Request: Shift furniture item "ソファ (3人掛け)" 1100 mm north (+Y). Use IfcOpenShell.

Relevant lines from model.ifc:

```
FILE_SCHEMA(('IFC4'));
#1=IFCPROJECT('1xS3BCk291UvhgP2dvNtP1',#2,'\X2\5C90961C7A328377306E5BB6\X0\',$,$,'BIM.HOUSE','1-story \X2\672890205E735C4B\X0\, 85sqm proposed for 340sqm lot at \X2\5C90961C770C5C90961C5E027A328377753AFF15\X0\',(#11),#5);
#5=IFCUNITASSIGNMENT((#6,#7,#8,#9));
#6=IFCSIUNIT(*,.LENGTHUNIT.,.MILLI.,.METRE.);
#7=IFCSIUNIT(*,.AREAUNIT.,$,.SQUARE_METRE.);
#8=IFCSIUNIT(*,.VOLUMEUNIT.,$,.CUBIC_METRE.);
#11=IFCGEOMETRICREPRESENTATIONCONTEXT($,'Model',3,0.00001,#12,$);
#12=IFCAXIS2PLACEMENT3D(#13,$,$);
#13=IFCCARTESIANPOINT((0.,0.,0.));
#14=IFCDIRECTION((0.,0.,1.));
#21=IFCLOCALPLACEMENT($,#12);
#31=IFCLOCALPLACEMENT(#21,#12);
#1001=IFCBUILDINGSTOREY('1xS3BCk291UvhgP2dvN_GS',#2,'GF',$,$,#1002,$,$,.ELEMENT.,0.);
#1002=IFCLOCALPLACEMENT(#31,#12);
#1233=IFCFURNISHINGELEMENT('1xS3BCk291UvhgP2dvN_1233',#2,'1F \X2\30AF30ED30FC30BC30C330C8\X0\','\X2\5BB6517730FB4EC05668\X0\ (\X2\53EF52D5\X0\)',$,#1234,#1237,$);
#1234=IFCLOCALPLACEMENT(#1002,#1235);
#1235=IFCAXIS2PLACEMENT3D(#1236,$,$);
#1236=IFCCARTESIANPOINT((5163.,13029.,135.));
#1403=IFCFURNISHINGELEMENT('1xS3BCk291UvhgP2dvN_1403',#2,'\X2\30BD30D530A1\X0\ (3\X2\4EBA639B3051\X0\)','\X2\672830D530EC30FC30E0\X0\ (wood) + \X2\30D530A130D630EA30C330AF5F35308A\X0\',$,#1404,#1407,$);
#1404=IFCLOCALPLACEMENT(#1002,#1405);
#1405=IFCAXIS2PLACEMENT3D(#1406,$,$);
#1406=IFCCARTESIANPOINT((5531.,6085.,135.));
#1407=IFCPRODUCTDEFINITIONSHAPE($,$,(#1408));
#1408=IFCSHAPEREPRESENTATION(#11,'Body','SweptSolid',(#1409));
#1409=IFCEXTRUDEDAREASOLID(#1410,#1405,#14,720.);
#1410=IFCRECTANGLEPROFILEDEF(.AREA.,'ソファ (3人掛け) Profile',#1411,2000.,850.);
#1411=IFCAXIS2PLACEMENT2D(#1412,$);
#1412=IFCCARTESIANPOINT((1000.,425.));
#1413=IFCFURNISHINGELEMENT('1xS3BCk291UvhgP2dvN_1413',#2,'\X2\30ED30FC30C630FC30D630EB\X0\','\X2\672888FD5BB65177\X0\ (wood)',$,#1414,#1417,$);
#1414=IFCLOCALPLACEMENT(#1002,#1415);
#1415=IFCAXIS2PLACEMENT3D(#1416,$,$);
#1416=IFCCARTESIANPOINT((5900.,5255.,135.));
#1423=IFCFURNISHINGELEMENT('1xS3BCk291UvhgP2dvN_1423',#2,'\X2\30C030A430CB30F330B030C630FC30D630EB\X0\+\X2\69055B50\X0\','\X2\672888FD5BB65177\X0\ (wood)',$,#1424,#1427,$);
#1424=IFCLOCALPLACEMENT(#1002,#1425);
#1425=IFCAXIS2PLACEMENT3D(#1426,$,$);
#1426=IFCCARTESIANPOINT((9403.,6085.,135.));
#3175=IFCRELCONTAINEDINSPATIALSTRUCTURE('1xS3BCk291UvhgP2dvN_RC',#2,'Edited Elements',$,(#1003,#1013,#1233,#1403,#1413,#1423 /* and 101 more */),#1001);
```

```python
import ifcopenshell
import ifcopenshell.api.geometry
import ifcopenshell.util.placement
import ifcopenshell.util.unit

model = ifcopenshell.open("model.ifc")
unit_scale = ifcopenshell.util.unit.calculate_unit_scale(model)

item = model.by_guid("1xS3BCk291UvhgP2dvN_1403")
matrix = ifcopenshell.util.placement.get_local_placement(item.ObjectPlacement)
matrix[1, 3] += 1.1 / unit_scale
ifcopenshell.api.geometry.edit_object_placement(model, product=item, matrix=matrix, is_si=False)

print(ifcopenshell.util.placement.get_local_placement(item.ObjectPlacement).round(3) + 0.0)

model.write("model_updated.ifc")
```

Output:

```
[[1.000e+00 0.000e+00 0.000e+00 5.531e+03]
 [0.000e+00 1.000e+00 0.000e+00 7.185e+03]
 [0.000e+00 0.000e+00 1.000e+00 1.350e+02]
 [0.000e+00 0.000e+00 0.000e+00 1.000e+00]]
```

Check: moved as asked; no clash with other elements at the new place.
